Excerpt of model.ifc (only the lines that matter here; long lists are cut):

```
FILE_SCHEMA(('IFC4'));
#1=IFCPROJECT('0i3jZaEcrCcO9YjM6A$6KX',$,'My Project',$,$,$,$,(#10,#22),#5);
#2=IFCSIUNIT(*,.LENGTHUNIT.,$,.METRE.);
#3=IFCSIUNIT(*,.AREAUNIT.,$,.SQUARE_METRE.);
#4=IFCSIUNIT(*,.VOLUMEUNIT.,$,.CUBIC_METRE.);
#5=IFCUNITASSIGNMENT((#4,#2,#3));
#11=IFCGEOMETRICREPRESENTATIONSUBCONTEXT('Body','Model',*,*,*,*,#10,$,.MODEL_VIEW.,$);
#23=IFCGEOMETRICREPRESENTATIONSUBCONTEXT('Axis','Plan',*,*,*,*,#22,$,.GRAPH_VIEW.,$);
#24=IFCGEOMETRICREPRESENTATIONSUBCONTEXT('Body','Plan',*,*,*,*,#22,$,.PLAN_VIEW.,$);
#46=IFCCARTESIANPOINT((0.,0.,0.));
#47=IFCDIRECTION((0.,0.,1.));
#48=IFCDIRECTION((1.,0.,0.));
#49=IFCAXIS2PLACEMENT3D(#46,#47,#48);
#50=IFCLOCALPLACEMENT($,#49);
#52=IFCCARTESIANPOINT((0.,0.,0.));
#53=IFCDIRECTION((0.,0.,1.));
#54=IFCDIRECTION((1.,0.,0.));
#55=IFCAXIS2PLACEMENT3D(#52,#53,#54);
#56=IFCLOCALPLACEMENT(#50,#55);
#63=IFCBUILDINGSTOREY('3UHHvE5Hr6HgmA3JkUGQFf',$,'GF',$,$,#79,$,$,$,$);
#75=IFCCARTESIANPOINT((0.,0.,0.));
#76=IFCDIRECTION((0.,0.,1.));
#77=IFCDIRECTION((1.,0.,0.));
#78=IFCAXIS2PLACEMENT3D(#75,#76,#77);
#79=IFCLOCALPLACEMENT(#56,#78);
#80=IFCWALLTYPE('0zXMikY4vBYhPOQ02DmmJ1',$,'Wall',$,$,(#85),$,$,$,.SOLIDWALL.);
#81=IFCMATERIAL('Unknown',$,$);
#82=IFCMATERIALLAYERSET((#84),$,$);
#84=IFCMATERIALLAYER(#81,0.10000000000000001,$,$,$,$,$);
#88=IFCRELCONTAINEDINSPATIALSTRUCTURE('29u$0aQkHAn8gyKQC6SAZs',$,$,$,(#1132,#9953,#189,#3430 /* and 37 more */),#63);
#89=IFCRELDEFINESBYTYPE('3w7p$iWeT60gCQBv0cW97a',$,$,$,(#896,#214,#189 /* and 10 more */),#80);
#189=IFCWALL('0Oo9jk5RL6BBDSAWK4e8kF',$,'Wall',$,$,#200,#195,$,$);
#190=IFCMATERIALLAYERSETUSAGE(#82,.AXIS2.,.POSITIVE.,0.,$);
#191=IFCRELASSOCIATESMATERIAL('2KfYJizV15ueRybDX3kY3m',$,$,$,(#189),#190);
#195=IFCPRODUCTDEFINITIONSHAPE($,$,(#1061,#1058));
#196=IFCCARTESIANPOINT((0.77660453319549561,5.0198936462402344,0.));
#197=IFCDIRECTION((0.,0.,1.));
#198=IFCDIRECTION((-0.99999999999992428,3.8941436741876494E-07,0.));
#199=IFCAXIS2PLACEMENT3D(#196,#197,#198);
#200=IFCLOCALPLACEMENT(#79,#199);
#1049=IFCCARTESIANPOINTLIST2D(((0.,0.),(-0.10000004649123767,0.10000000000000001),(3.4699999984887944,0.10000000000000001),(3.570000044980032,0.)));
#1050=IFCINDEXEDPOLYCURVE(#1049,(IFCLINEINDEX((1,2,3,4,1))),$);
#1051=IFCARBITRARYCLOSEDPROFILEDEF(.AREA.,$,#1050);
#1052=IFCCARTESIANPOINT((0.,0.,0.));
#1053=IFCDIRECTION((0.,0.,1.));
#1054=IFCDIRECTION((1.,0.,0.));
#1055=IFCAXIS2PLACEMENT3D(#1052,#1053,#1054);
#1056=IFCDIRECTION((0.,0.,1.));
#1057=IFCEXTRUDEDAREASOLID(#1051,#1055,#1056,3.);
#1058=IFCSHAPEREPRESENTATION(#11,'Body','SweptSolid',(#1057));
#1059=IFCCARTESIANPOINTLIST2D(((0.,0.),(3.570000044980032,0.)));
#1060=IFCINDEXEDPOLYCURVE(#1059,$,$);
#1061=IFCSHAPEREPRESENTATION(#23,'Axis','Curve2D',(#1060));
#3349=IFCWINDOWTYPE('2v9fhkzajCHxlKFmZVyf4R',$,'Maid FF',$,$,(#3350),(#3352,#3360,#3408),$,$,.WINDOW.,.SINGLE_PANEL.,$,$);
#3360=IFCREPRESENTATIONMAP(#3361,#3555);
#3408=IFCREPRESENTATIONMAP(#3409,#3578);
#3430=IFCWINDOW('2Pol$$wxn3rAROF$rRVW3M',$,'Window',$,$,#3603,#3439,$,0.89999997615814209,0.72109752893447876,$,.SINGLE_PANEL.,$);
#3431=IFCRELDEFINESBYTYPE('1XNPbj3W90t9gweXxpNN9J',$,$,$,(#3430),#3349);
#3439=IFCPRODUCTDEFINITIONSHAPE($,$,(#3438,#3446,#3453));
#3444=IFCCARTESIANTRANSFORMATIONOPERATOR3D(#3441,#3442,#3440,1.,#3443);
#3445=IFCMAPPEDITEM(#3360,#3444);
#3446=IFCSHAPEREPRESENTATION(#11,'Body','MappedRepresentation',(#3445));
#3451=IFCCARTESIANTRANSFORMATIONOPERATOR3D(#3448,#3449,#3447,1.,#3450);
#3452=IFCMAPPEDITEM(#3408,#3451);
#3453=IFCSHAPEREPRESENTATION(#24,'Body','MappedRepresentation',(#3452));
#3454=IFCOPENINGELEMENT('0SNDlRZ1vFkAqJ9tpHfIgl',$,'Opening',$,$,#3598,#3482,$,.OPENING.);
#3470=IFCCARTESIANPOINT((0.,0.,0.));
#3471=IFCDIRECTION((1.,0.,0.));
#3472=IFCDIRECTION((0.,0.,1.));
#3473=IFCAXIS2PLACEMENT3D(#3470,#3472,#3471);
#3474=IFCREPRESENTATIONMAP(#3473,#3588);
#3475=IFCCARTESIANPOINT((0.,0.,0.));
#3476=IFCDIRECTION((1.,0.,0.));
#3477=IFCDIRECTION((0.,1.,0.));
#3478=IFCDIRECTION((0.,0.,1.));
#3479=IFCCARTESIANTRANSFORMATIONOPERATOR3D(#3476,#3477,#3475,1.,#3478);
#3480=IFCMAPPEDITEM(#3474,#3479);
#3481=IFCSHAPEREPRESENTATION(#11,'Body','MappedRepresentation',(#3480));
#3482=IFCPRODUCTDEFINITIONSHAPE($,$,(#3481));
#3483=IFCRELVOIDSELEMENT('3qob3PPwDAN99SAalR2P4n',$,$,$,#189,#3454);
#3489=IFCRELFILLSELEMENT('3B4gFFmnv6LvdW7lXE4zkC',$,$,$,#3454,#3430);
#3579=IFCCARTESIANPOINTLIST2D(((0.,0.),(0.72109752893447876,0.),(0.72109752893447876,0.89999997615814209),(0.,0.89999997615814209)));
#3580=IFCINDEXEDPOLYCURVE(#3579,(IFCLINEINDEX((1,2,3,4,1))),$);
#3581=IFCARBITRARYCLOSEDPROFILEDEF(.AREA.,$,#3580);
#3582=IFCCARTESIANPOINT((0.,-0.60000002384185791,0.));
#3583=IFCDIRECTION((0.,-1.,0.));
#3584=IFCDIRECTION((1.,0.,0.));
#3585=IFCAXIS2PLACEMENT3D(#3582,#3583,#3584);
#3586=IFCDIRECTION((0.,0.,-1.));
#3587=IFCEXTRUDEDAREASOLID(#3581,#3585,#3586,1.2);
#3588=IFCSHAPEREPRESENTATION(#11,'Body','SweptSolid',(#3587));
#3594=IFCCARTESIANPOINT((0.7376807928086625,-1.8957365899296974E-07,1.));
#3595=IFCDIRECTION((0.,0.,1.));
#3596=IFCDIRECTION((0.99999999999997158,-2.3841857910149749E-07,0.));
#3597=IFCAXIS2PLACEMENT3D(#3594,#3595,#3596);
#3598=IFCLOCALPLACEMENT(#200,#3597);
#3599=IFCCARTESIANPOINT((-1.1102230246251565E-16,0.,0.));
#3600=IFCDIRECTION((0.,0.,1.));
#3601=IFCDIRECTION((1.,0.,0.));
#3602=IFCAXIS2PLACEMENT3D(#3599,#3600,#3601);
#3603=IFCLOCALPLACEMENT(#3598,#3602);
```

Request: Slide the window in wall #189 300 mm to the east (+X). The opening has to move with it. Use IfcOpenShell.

```python
import ifcopenshell
import ifcopenshell.api.geometry
import ifcopenshell.util.placement

model = ifcopenshell.open("model.ifc")

window = model.by_guid("2Pol$$wxn3rAROF$rRVW3M")
opening = window.FillsVoids[0].RelatingOpeningElement
wall = opening.VoidsElements[0].RelatingBuildingElement

wall_matrix = ifcopenshell.util.placement.get_local_placement(wall.ObjectPlacement)
shift = wall_matrix[:3, 0] * -0.3
before = ifcopenshell.util.placement.get_local_placement(window.ObjectPlacement)[:3, 3].copy()

# The window is placed relative to its opening, so it follows when the opening moves.
matrix = ifcopenshell.util.placement.get_local_placement(opening.ObjectPlacement)
matrix[:3, 3] += shift
ifcopenshell.api.geometry.edit_object_placement(
    model, product=opening, matrix=matrix, is_si=False, should_transform_children=True
)

after = ifcopenshell.util.placement.get_local_placement(window.ObjectPlacement)[:3, 3]
print("window moved by", (after - before).round(3) + 0.0)

model.write("model_rev.ifc")
```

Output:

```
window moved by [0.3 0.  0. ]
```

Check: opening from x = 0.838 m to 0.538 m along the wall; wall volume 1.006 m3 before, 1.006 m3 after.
